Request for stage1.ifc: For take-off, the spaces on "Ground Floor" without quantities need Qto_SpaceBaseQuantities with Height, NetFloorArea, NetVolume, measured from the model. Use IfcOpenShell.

First a look at what the model holds.

```python
import ifcopenshell
import ifcopenshell.util.element
import ifcopenshell.util.unit

model = ifcopenshell.open("stage1.ifc")
print(model.schema)
for unit_type in ("LENGTHUNIT", "AREAUNIT", "VOLUMEUNIT"):
    print(unit_type, ifcopenshell.util.unit.calculate_unit_scale(model, unit_type))
storey = next(s for s in model.by_type("IfcBuildingStorey") if s.Name == "Ground Floor")
spaces = [e for e in ifcopenshell.util.element.get_decomposition(storey) if e.is_a("IfcSpace")]
for e in sorted(spaces, key=lambda e: e.id()):
    print(e.id(), e.is_a(), e.Name, list(ifcopenshell.util.element.get_psets(e, qtos_only=True)), sep=" | ")
```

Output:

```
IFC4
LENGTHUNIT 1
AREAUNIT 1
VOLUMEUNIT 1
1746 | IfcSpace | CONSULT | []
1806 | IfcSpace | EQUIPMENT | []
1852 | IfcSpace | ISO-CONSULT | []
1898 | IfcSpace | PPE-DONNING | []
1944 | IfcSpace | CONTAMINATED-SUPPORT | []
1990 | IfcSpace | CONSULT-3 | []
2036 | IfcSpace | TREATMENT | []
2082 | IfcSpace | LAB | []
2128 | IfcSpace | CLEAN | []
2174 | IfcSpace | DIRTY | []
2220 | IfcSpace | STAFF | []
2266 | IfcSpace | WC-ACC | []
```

```python
import ifcopenshell
import ifcopenshell.api.pset
import ifcopenshell.geom
import ifcopenshell.util.element
import ifcopenshell.util.shape
import ifcopenshell.util.unit

model = ifcopenshell.open("stage1.ifc")
unit_scale = ifcopenshell.util.unit.calculate_unit_scale(model)
area_scale = ifcopenshell.util.unit.calculate_unit_scale(model, "AREAUNIT")
volume_scale = ifcopenshell.util.unit.calculate_unit_scale(model, "VOLUMEUNIT")
settings = ifcopenshell.geom.settings()

storey = next(s for s in model.by_type("IfcBuildingStorey") if s.Name == "Ground Floor")
spaces = [e for e in ifcopenshell.util.element.get_decomposition(storey) if e.is_a("IfcSpace")]

for e in sorted(spaces, key=lambda e: e.id()):
    if ifcopenshell.util.element.get_psets(e, qtos_only=True, should_inherit=False):
        continue
    # Geometry comes back in metres, in the element's own axes.
    shape = ifcopenshell.geom.create_shape(settings, e)
    values = {
        "Height": ifcopenshell.util.shape.get_z(shape.geometry) / unit_scale,
        "NetFloorArea": ifcopenshell.util.shape.get_footprint_area(shape.geometry) / area_scale,
        "NetVolume": ifcopenshell.util.shape.get_volume(shape.geometry) / volume_scale,
    }
    qto = ifcopenshell.api.pset.add_qto(model, product=e, name="Qto_SpaceBaseQuantities")
    ifcopenshell.api.pset.edit_qto(model, qto=qto, properties=values)
    print(e.id(), {k: round(v, 3) for k, v in values.items()})

model.write("stage1_v2.ifc")
```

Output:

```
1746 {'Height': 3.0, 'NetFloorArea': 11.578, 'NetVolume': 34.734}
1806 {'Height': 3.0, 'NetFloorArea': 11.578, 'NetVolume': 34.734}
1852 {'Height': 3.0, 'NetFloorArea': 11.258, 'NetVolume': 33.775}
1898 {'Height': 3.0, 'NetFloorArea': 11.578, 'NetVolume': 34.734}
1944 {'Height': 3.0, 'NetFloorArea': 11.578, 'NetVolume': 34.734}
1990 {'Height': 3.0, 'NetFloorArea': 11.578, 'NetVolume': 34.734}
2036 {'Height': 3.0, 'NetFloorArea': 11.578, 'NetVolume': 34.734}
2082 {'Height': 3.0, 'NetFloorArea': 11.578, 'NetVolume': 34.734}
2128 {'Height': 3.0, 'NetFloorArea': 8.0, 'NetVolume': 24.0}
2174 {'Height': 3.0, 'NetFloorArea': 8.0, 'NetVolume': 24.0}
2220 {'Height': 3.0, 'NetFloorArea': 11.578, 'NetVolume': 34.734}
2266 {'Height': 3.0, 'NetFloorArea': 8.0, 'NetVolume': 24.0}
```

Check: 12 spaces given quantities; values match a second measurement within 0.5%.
